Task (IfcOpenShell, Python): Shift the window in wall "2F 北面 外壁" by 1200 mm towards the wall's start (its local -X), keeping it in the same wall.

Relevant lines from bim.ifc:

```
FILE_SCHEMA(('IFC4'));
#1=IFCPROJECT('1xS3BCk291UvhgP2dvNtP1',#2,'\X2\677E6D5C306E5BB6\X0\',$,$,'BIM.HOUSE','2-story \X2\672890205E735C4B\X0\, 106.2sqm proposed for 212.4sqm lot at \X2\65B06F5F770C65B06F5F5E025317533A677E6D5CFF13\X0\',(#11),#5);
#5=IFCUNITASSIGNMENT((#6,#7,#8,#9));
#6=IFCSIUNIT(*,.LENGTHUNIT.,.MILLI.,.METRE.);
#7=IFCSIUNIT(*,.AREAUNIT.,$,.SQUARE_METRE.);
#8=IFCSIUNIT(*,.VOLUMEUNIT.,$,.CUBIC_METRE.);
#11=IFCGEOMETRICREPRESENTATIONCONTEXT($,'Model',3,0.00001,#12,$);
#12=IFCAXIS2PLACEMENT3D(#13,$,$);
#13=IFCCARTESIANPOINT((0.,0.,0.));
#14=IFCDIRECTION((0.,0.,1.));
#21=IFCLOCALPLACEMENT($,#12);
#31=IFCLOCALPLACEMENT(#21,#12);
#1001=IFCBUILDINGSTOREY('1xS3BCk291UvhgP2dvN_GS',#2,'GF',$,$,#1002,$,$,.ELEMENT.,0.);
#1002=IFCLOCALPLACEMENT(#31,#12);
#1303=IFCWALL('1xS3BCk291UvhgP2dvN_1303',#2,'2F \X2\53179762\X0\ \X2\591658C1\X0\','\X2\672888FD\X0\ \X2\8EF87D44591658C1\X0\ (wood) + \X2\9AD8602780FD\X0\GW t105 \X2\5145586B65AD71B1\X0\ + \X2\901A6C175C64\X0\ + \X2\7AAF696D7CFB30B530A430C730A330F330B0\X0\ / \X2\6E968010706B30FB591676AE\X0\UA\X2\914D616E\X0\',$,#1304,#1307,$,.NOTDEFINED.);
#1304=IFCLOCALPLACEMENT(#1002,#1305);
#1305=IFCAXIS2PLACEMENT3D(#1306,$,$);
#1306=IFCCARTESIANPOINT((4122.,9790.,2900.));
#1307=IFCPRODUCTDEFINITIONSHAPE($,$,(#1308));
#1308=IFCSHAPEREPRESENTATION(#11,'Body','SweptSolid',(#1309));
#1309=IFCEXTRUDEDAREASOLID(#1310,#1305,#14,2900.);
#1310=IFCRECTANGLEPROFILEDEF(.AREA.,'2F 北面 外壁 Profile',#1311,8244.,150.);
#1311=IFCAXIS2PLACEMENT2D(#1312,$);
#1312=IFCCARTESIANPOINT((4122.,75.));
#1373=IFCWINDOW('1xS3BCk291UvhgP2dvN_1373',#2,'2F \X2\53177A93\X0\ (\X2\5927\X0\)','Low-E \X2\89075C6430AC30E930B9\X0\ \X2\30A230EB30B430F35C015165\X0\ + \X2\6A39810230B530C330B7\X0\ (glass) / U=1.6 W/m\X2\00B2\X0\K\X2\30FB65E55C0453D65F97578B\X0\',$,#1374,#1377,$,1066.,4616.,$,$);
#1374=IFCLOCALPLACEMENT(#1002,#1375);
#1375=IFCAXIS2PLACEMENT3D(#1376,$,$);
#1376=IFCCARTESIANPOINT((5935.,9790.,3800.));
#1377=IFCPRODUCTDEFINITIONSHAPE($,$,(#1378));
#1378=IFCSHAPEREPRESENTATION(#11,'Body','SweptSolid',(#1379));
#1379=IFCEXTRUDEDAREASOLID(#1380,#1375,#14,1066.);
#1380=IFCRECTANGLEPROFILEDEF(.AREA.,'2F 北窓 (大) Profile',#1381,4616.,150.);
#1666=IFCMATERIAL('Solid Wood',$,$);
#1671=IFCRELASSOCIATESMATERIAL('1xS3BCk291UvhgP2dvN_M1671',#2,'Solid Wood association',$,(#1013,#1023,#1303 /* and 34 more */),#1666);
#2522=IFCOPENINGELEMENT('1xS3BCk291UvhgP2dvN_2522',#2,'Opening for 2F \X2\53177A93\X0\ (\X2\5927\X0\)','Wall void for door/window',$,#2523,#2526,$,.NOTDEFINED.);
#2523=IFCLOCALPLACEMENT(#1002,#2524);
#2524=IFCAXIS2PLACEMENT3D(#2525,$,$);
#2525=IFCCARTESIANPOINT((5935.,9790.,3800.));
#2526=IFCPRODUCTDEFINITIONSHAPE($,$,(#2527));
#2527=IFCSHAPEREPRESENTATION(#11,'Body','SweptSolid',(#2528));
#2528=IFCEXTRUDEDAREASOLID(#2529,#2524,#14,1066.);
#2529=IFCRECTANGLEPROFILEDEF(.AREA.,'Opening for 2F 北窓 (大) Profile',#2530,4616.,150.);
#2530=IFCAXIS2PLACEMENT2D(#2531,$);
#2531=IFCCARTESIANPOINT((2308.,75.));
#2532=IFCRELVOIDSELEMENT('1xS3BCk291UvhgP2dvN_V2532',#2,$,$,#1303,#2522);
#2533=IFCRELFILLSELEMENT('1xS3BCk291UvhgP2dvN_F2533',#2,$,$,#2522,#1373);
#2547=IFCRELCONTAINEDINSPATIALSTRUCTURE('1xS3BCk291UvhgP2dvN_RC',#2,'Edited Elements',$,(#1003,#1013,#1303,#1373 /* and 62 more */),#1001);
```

```python
import ifcopenshell
import ifcopenshell.api.geometry
import ifcopenshell.util.placement
import ifcopenshell.util.unit

model = ifcopenshell.open("bim.ifc")
unit_scale = ifcopenshell.util.unit.calculate_unit_scale(model)

window = model.by_guid("1xS3BCk291UvhgP2dvN_1373")
opening = window.FillsVoids[0].RelatingOpeningElement
wall = opening.VoidsElements[0].RelatingBuildingElement

wall_matrix = ifcopenshell.util.placement.get_local_placement(wall.ObjectPlacement)
shift = wall_matrix[:3, 0] * -1.2 / unit_scale
before = ifcopenshell.util.placement.get_local_placement(window.ObjectPlacement)[:3, 3].copy()

# The window is not placed relative to its opening, so move both.
for product in (opening, window):
    matrix = ifcopenshell.util.placement.get_local_placement(product.ObjectPlacement)
    matrix[:3, 3] += shift
    ifcopenshell.api.geometry.edit_object_placement(model, product=product, matrix=matrix, is_si=False)

after = ifcopenshell.util.placement.get_local_placement(window.ObjectPlacement)[:3, 3]
print("window moved by", (after - before).round(3) + 0.0)

model.write("bim-out.ifc")
```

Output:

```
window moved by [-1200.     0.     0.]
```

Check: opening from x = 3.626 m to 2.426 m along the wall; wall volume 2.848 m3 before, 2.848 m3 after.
